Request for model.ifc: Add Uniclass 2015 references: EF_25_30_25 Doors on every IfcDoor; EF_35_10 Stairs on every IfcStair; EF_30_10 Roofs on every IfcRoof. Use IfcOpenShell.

First a look at what the model holds.

```python
import ifcopenshell

model = ifcopenshell.open("model.ifc")
print(model.schema)
print("classifications:", [c.Name for c in model.by_type("IfcClassification")])
for ifc_class in ("IfcDoor", "IfcRoof", "IfcStair", "IfcWall", "IfcWindow"):
    print(ifc_class, len(model.by_type(ifc_class)))
```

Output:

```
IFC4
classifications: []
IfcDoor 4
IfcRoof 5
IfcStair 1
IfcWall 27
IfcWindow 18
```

```python
import ifcopenshell
import ifcopenshell.api.classification

model = ifcopenshell.open("model.ifc")

system = ifcopenshell.api.classification.add_classification(model, classification="Uniclass 2015")

codes = {
    "IfcDoor": ("EF_25_30_25", "Doors"),
    "IfcStair": ("EF_35_10", "Stairs"),
    "IfcRoof": ("EF_30_10", "Roofs"),
}
for ifc_class, (code, name) in codes.items():
    products = model.by_type(ifc_class)
    ifcopenshell.api.classification.add_reference(
        model, products=products, classification=system, identification=code, name=name
    )
    print(code, len(products))

model.write("model_edited.ifc")
```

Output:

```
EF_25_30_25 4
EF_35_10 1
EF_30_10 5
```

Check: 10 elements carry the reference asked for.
